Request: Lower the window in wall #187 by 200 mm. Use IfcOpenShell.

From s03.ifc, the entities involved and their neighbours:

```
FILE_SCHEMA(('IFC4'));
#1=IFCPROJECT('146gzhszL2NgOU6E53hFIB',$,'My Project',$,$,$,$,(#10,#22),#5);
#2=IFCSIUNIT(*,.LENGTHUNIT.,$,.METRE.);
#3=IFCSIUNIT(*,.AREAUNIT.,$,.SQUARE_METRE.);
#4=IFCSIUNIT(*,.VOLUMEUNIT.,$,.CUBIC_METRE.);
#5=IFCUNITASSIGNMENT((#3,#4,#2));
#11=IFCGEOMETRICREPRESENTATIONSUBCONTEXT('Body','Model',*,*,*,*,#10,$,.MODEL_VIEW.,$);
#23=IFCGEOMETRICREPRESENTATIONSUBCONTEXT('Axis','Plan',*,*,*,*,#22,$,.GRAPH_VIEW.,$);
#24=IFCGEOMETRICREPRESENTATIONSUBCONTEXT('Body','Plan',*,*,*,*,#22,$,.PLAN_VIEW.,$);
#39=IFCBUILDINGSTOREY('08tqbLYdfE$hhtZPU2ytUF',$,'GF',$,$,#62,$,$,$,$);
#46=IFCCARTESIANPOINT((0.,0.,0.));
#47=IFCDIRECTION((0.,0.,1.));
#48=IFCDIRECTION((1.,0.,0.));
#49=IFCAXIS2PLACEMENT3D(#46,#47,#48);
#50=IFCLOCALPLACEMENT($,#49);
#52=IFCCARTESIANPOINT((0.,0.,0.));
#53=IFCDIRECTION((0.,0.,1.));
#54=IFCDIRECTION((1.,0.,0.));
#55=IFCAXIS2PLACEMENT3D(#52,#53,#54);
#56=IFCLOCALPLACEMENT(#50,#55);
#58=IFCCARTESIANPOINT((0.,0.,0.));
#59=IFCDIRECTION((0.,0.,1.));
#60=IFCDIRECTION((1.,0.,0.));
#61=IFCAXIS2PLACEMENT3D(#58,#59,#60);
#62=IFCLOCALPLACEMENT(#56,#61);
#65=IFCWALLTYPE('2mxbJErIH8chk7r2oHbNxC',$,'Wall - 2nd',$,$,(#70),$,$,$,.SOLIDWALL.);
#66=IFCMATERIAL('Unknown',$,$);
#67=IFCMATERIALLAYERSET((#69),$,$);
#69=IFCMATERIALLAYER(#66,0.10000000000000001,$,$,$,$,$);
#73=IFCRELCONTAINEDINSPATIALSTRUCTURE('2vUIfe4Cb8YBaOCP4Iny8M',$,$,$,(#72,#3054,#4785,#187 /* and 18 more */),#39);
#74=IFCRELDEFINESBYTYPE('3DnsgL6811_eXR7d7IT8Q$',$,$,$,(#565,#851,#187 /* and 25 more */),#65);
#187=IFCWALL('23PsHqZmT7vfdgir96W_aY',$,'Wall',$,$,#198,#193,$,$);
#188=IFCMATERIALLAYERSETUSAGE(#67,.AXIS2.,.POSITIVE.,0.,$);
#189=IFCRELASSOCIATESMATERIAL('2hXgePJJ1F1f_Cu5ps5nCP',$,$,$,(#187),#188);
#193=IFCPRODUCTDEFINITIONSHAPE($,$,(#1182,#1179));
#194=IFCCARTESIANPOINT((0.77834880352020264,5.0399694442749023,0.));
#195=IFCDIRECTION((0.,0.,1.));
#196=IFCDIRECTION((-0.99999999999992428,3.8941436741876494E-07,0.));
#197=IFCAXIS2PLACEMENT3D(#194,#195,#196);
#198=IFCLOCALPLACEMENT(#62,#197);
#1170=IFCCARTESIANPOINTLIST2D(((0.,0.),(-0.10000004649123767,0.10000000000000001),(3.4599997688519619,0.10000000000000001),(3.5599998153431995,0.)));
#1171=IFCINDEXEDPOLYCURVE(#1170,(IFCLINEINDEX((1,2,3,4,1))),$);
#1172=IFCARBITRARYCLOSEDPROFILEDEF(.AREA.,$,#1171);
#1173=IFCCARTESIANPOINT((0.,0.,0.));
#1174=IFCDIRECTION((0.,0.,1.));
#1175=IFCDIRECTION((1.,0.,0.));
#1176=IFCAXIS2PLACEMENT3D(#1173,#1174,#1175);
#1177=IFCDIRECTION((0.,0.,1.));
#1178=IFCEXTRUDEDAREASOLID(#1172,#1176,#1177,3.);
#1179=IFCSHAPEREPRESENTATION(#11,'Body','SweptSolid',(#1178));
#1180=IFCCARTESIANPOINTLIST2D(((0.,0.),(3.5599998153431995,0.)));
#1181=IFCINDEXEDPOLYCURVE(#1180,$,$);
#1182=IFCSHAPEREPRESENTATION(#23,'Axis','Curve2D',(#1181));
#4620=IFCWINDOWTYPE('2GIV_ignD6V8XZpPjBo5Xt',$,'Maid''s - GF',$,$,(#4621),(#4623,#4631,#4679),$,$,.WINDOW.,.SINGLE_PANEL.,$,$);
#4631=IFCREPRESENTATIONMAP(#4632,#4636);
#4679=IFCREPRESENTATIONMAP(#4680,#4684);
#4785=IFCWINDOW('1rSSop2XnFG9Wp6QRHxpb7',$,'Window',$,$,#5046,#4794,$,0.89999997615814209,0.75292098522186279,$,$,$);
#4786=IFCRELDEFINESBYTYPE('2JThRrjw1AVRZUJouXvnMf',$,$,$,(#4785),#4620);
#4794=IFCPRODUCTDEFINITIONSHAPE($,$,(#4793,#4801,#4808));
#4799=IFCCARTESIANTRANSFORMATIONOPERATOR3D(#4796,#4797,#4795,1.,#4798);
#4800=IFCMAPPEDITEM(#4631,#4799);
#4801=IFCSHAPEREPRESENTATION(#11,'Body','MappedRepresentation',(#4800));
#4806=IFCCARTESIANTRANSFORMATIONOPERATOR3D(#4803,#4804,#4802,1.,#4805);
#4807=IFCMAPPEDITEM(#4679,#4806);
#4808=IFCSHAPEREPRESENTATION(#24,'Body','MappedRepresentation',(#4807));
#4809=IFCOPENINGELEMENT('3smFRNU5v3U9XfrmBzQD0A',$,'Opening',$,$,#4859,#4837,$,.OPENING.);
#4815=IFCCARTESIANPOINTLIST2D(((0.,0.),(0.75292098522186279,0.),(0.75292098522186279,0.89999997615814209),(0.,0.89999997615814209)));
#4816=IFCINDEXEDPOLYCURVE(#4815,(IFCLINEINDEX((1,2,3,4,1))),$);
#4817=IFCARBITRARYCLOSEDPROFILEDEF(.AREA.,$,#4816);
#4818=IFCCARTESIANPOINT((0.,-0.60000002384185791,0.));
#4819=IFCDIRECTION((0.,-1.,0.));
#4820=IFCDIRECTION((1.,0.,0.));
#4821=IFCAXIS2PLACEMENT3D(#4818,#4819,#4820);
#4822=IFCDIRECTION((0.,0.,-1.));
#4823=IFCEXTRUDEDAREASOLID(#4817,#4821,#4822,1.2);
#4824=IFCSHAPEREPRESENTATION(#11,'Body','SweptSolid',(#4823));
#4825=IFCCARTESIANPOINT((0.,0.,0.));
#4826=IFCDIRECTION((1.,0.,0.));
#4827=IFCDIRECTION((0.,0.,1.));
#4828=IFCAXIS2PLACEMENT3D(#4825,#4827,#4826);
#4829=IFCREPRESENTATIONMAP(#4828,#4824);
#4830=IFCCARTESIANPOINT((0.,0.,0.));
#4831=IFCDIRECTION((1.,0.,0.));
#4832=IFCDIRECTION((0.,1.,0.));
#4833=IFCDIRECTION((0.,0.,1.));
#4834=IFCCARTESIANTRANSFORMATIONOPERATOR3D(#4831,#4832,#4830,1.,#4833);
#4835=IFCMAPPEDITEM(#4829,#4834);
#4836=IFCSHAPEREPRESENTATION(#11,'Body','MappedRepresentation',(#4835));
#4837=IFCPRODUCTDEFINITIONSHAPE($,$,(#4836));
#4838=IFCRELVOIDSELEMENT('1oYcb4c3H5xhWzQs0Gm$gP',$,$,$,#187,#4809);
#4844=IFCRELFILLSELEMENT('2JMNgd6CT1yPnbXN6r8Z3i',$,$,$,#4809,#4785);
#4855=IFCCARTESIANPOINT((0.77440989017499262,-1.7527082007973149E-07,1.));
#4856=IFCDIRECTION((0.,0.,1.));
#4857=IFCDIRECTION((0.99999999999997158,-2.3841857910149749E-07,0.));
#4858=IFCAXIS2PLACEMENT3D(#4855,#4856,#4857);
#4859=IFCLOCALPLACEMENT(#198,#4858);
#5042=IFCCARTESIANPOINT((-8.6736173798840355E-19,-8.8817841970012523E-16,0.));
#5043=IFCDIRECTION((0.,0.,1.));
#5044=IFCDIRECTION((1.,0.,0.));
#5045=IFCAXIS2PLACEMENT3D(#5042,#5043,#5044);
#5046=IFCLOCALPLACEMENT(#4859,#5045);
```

```python
import numpy as np
import ifcopenshell
import ifcopenshell.api.geometry
import ifcopenshell.util.placement
import ifcopenshell.util.unit

model = ifcopenshell.open("s03.ifc")
unit_scale = ifcopenshell.util.unit.calculate_unit_scale(model)

window = model.by_guid("1rSSop2XnFG9Wp6QRHxpb7")
opening = window.FillsVoids[0].RelatingOpeningElement
dz = -0.2

shift = np.array([0.0, 0.0, dz])
# The window is placed relative to its opening, so it follows when the opening moves.
matrix = ifcopenshell.util.placement.get_local_placement(opening.ObjectPlacement)
matrix[:3, 3] += shift
ifcopenshell.api.geometry.edit_object_placement(
    model, product=opening, matrix=matrix, is_si=False, should_transform_children=True
)

print(f"moved by {dz * unit_scale:+.3f} m")

model.write("s03_updated.ifc")
```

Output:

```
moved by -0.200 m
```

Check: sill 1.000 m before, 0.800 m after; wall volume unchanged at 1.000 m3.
